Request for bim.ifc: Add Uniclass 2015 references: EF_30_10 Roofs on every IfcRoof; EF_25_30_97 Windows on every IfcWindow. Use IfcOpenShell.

First a look at what the model holds.

```python
import ifcopenshell

model = ifcopenshell.open("bim.ifc")
print(model.schema)
print("classifications:", [c.Name for c in model.by_type("IfcClassification")])
for ifc_class in ("IfcDoor", "IfcRoof", "IfcStair", "IfcWall", "IfcWindow"):
    print(ifc_class, len(model.by_type(ifc_class)))
```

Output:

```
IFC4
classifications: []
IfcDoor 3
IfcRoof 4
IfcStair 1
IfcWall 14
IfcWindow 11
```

```python
import ifcopenshell
import ifcopenshell.api.classification

model = ifcopenshell.open("bim.ifc")

system = ifcopenshell.api.classification.add_classification(model, classification="Uniclass 2015")

codes = {
    "IfcRoof": ("EF_30_10", "Roofs"),
    "IfcWindow": ("EF_25_30_97", "Windows"),
}
for ifc_class, (code, name) in codes.items():
    products = model.by_type(ifc_class)
    ifcopenshell.api.classification.add_reference(
        model, products=products, classification=system, identification=code, name=name
    )
    print(code, len(products))

model.write("bim-out.ifc")
```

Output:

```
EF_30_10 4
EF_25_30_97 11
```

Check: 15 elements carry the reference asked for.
